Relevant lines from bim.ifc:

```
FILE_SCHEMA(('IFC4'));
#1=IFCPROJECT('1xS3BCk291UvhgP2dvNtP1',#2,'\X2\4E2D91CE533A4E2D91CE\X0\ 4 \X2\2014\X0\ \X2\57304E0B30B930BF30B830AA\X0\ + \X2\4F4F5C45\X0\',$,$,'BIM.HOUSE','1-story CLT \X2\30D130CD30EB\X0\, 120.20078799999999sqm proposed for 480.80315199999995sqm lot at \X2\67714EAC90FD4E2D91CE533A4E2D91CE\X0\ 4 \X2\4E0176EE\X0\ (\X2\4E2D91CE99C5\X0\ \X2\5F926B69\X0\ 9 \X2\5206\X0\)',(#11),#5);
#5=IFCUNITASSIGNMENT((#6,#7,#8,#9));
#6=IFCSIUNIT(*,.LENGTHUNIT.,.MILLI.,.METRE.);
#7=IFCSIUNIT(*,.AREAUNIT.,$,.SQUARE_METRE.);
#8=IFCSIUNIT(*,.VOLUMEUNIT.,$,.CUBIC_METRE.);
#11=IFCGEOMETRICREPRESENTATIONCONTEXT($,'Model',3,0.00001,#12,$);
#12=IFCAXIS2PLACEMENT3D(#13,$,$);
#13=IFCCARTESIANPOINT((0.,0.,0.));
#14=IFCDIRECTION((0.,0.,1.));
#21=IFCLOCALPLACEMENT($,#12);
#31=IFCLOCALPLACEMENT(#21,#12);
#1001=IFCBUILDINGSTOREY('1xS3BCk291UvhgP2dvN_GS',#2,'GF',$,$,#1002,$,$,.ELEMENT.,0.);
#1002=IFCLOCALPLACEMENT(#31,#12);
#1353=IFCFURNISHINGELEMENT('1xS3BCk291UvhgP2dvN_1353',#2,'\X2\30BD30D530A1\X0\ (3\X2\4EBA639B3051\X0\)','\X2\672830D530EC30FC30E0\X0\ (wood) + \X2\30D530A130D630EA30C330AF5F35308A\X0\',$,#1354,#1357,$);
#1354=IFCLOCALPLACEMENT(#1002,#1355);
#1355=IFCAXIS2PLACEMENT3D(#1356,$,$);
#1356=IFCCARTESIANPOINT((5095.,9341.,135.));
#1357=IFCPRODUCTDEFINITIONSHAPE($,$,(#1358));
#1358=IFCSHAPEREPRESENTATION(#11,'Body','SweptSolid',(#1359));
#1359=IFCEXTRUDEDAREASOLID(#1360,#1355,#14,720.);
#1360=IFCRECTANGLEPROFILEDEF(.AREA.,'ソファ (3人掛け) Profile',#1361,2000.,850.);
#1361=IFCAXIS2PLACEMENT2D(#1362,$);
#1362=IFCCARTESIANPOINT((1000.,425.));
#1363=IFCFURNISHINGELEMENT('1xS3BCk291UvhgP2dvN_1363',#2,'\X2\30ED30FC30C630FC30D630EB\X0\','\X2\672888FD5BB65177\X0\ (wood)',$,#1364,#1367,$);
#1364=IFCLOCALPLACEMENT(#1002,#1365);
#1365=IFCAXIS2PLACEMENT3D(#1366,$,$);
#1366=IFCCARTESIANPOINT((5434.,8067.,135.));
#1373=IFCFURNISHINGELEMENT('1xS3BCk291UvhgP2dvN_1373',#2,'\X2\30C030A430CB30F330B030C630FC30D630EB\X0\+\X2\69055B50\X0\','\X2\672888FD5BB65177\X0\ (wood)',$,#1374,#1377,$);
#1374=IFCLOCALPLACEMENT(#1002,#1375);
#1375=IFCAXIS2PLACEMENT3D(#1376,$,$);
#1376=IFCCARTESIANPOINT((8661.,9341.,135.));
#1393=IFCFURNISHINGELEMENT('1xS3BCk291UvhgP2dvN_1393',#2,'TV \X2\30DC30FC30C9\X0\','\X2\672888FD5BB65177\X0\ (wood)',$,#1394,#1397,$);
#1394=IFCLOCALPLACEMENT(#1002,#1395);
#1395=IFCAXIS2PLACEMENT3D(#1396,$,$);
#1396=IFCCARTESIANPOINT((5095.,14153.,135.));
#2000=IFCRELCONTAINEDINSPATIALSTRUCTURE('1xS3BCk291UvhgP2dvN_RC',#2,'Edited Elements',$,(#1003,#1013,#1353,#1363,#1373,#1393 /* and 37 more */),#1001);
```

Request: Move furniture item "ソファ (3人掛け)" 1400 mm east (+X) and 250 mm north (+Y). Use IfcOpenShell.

```python
import ifcopenshell
import ifcopenshell.api.geometry
import ifcopenshell.util.placement

model = ifcopenshell.open("bim.ifc")

item = model.by_guid("1xS3BCk291UvhgP2dvN_1353")
matrix = ifcopenshell.util.placement.get_local_placement(item.ObjectPlacement)
matrix[0, 3] += 1400.0
matrix[1, 3] += 250.0
ifcopenshell.api.geometry.edit_object_placement(model, product=item, matrix=matrix, is_si=False)

print(ifcopenshell.util.placement.get_local_placement(item.ObjectPlacement).round(3) + 0.0)

model.write("bim_rev.ifc")
```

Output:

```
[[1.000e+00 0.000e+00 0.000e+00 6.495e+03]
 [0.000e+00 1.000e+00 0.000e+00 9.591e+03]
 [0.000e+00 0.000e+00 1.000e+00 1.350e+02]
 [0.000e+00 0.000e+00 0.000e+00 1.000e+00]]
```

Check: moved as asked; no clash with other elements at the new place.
